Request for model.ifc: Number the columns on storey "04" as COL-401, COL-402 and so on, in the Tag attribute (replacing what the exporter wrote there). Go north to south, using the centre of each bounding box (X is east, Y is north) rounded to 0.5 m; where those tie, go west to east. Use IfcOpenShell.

First a look at what the model holds.

```python
import ifcopenshell
import ifcopenshell.util.element
import ifcopenshell.util.placement

model = ifcopenshell.open("model.ifc")
print(model.schema)
storey = next(s for s in model.by_type("IfcBuildingStorey") if s.Name == "04")
columns = [e for e in ifcopenshell.util.element.get_decomposition(storey) if e.is_a("IfcColumn")]
for e in sorted(columns, key=lambda e: e.id()):
    origin = ifcopenshell.util.placement.get_local_placement(e.ObjectPlacement)[:3, 3]
    print(e.id(), e.Tag, e.Name, origin.round(2) + 0.0, sep=" | ")
```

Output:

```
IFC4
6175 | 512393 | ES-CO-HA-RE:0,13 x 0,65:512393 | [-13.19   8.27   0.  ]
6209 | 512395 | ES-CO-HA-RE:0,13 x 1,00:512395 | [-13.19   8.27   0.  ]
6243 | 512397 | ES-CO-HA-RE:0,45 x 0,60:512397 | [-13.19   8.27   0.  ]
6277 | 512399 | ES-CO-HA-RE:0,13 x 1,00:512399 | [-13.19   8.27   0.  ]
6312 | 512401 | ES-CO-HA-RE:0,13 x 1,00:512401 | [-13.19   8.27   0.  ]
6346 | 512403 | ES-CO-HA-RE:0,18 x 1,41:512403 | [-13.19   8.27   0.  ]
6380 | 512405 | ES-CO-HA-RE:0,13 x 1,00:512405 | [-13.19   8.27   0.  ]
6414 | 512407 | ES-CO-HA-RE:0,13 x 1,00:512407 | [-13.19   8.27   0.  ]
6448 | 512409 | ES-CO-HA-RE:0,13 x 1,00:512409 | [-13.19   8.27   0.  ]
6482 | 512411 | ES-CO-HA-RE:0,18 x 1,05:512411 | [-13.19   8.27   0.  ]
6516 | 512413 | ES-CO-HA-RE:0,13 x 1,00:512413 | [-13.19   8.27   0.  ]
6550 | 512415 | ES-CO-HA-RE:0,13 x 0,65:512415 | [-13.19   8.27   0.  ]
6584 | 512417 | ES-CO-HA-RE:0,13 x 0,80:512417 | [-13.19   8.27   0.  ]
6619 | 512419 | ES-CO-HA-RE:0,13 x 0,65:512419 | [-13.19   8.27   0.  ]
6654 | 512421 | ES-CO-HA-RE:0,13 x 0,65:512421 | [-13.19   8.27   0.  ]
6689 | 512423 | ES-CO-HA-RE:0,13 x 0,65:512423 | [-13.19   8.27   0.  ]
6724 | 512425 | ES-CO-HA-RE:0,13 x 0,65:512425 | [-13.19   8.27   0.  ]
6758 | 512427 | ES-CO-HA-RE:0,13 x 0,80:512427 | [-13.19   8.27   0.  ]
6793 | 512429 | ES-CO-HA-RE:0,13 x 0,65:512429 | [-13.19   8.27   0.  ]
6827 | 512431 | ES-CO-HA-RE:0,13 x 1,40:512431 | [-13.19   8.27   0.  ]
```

```python
import ifcopenshell
import ifcopenshell.geom
import ifcopenshell.util.element
import ifcopenshell.util.shape

model = ifcopenshell.open("model.ifc")
settings = ifcopenshell.geom.settings()
settings.set("use-world-coords", True)


def centre(element):
    shape = ifcopenshell.geom.create_shape(settings, element)
    return ifcopenshell.util.shape.get_bbox_centroid(shape.geometry)


storey = next(s for s in model.by_type("IfcBuildingStorey") if s.Name == "04")
columns = [e for e in ifcopenshell.util.element.get_decomposition(storey) if e.is_a("IfcColumn")]

# Insertion points can sit at a corner or the storey origin, so sort by the geometry (in metres).
centres = {e: centre(e) for e in columns}
columns.sort(key=lambda e: (-round(centres[e][1] / 0.5), centres[e][0]))

for i, e in enumerate(columns, start=1):
    number = f"COL-4{i:02d}"
    e.Tag = number
    print(e.id(), number)

model.write("model-out.ifc")
```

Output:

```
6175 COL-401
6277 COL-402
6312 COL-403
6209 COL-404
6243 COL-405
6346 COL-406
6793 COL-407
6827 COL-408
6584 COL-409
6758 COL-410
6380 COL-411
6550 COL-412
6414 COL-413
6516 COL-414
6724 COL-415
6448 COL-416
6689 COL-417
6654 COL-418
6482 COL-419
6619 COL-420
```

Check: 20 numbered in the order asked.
